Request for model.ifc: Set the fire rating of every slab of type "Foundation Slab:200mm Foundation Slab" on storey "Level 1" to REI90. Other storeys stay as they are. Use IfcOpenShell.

First a look at what the model holds.

```python
import ifcopenshell
import ifcopenshell.util.element

model = ifcopenshell.open("model.ifc")
print(model.schema)
storey = next(s for s in model.by_type("IfcBuildingStorey") if s.Name == "Level 1")
slabs = [e for e in ifcopenshell.util.element.get_decomposition(storey) if e.is_a("IfcSlab")]
seen = {}
for e in slabs:
    element_type = ifcopenshell.util.element.get_type(e)
    key = (element_type.Name if element_type != e and element_type else None, ifcopenshell.util.element.get_pset(e, "Pset_SlabCommon", "FireRating"))
    seen[key] = seen.get(key, 0) + 1
for (name, value), count in sorted(seen.items(), key=str):
    print(count, "x", name, "|", value)
```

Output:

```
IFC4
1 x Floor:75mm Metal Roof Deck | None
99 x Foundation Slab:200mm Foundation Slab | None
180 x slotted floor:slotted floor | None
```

```python
import ifcopenshell
import ifcopenshell.api.pset
import ifcopenshell.util.element

model = ifcopenshell.open("model.ifc")

storey = next(s for s in model.by_type("IfcBuildingStorey") if s.Name == "Level 1")
slabs = [e for e in ifcopenshell.util.element.get_decomposition(storey) if e.is_a("IfcSlab")]

count = 0
for e in slabs:
    element_type = ifcopenshell.util.element.get_type(e)
    if element_type in (None, e) or element_type.Name != "Foundation Slab:200mm Foundation Slab":
        continue
    # add_pset returns the element's existing set when there is one.
    pset = ifcopenshell.api.pset.add_pset(model, product=e, name="Pset_SlabCommon")
    ifcopenshell.api.pset.edit_pset(model, pset=pset, properties={"FireRating": "REI90"})
    count += 1

print(count, "slabs updated")

model.write("model-out.ifc")
```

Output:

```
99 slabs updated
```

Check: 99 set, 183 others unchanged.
